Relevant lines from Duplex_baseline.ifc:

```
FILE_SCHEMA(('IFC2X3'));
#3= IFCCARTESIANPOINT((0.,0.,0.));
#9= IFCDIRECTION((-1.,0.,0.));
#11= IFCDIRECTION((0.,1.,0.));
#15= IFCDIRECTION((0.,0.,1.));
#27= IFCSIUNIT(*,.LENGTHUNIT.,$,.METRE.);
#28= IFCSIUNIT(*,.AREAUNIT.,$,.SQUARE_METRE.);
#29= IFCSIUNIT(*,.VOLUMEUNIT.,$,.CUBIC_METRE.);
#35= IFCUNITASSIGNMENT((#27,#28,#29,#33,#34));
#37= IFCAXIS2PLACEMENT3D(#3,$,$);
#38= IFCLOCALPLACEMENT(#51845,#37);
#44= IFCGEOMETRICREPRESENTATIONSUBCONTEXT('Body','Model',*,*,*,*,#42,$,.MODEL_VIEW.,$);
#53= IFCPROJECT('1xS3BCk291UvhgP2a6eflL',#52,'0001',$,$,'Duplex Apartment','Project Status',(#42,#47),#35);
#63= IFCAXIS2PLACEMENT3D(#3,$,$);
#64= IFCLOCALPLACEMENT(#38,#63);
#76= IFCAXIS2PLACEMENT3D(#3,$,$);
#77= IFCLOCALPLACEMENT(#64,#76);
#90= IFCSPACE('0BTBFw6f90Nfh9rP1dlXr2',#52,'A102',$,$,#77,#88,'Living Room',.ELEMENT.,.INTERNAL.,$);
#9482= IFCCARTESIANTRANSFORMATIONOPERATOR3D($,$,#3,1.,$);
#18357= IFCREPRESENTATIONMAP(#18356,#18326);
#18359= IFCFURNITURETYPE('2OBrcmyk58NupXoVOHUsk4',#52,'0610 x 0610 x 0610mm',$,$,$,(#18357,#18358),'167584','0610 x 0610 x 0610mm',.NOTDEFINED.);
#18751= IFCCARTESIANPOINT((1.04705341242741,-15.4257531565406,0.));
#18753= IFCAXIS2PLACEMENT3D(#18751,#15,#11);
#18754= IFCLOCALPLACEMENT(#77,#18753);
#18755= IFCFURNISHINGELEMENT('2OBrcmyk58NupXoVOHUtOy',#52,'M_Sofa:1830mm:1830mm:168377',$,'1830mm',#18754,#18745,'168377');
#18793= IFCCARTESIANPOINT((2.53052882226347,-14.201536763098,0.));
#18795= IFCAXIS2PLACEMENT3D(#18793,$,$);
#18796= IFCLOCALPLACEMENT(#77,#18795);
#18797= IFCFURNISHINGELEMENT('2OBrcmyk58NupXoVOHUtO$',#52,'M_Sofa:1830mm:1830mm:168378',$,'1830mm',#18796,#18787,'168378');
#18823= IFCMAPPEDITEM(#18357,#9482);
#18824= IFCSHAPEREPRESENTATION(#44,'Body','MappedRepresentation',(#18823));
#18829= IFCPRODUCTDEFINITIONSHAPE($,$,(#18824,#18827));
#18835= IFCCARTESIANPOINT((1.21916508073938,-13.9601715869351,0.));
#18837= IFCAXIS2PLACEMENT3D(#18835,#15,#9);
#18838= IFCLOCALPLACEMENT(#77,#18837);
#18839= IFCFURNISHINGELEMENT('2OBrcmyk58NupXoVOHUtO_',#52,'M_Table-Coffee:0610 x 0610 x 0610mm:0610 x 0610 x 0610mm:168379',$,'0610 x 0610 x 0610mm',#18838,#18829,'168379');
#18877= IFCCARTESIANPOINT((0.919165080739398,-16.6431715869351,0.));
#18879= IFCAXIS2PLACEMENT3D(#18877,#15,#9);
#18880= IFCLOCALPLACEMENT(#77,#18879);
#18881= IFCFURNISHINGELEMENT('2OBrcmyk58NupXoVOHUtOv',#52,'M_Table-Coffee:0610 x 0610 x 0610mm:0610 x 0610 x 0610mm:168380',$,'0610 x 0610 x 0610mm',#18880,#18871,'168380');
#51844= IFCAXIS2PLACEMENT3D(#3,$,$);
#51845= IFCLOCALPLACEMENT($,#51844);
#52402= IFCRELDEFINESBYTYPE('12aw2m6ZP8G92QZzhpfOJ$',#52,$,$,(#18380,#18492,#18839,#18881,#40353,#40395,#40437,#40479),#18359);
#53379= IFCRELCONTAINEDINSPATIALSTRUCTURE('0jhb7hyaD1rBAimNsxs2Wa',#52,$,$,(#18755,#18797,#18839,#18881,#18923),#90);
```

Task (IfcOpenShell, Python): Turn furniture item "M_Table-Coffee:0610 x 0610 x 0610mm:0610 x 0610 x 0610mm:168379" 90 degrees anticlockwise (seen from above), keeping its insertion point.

```python
import ifcopenshell
import ifcopenshell.api.geometry
import ifcopenshell.util.placement

model = ifcopenshell.open("Duplex_baseline.ifc")

item = model.by_guid("2OBrcmyk58NupXoVOHUtO_")
matrix = ifcopenshell.util.placement.get_local_placement(item.ObjectPlacement)
matrix = matrix @ ifcopenshell.util.placement.rotation(90, "Z")
ifcopenshell.api.geometry.edit_object_placement(model, product=item, matrix=matrix, is_si=False)

print(ifcopenshell.util.placement.get_local_placement(item.ObjectPlacement).round(3) + 0.0)

model.write("Duplex_baseline_v2.ifc")
```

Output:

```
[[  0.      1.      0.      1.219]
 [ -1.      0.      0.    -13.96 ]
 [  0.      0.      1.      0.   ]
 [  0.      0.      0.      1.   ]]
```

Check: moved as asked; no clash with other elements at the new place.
